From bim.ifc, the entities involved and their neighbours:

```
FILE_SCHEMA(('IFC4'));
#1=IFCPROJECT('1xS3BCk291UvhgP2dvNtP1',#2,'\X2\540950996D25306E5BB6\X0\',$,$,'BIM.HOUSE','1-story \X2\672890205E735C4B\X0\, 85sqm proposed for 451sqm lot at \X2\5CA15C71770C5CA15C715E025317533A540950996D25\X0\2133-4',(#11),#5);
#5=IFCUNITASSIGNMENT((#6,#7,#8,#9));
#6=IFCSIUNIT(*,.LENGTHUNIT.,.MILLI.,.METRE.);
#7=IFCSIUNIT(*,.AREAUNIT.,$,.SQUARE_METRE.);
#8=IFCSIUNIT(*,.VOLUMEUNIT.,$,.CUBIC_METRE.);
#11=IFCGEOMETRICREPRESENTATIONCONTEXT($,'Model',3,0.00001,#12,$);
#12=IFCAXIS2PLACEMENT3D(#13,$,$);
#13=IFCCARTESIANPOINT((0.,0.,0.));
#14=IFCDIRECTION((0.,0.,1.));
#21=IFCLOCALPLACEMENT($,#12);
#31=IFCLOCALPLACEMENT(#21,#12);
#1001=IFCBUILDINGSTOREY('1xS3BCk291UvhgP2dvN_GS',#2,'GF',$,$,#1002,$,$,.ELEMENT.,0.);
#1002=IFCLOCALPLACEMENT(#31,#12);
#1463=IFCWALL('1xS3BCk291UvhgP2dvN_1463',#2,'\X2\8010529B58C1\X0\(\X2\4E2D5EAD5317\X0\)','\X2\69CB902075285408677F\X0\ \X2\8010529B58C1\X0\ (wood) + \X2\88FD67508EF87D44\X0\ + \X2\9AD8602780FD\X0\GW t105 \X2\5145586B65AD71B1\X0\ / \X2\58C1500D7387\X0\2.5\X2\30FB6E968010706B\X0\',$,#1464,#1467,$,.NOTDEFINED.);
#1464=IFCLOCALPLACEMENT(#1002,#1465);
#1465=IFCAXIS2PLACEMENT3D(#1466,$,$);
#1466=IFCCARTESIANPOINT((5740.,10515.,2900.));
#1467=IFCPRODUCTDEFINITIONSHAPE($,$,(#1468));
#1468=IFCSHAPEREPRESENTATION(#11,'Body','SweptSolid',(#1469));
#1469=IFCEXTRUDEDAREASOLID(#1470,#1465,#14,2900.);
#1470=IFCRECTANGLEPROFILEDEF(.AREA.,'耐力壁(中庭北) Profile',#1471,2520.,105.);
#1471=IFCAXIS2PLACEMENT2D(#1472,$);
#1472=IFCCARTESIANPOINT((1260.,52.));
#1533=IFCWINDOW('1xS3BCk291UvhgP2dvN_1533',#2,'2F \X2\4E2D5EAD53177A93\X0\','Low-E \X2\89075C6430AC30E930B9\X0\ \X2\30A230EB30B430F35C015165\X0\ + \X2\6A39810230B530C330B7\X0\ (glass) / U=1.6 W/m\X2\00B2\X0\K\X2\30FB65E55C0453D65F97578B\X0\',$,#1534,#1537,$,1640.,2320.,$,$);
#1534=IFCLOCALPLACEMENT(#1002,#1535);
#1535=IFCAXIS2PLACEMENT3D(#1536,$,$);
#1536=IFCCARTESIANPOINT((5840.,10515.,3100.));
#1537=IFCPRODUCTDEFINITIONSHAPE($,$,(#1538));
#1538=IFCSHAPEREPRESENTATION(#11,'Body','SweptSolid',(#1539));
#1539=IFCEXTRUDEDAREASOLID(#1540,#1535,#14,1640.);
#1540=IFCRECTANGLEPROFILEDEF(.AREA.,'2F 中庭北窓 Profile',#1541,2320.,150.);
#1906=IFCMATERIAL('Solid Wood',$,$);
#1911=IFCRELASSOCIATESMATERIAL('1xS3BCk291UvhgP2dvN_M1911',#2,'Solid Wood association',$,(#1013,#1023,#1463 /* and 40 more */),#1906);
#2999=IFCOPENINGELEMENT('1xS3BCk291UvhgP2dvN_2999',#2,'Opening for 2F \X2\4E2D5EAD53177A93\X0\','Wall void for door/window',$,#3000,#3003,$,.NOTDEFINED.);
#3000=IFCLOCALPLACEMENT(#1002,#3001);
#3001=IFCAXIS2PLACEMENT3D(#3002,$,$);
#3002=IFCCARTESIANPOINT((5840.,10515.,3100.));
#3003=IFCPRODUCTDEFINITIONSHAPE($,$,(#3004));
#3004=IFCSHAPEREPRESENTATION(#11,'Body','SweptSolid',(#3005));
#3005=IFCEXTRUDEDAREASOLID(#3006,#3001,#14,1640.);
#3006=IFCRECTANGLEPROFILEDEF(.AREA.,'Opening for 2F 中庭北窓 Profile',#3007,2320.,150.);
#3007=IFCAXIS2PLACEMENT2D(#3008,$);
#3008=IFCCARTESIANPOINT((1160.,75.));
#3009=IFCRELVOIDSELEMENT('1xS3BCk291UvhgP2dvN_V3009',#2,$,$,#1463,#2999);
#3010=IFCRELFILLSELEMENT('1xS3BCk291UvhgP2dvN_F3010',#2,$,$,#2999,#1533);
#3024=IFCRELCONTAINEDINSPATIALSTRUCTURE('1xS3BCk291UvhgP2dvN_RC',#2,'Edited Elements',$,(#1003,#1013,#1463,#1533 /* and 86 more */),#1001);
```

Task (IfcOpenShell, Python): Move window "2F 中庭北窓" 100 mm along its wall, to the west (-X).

```python
import ifcopenshell
import ifcopenshell.api.geometry
import ifcopenshell.util.placement
import ifcopenshell.util.unit

model = ifcopenshell.open("bim.ifc")
unit_scale = ifcopenshell.util.unit.calculate_unit_scale(model)

window = model.by_guid("1xS3BCk291UvhgP2dvN_1533")
opening = window.FillsVoids[0].RelatingOpeningElement
wall = opening.VoidsElements[0].RelatingBuildingElement

wall_matrix = ifcopenshell.util.placement.get_local_placement(wall.ObjectPlacement)
shift = wall_matrix[:3, 0] * -0.1 / unit_scale
before = ifcopenshell.util.placement.get_local_placement(window.ObjectPlacement)[:3, 3].copy()

# The window is not placed relative to its opening, so move both.
for product in (opening, window):
    matrix = ifcopenshell.util.placement.get_local_placement(product.ObjectPlacement)
    matrix[:3, 3] += shift
    ifcopenshell.api.geometry.edit_object_placement(model, product=product, matrix=matrix, is_si=False)

after = ifcopenshell.util.placement.get_local_placement(window.ObjectPlacement)[:3, 3]
print("window moved by", (after - before).round(3) + 0.0)

model.write("bim-out.ifc")
```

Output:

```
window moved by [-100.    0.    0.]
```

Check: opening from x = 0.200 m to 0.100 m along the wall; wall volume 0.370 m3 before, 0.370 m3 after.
